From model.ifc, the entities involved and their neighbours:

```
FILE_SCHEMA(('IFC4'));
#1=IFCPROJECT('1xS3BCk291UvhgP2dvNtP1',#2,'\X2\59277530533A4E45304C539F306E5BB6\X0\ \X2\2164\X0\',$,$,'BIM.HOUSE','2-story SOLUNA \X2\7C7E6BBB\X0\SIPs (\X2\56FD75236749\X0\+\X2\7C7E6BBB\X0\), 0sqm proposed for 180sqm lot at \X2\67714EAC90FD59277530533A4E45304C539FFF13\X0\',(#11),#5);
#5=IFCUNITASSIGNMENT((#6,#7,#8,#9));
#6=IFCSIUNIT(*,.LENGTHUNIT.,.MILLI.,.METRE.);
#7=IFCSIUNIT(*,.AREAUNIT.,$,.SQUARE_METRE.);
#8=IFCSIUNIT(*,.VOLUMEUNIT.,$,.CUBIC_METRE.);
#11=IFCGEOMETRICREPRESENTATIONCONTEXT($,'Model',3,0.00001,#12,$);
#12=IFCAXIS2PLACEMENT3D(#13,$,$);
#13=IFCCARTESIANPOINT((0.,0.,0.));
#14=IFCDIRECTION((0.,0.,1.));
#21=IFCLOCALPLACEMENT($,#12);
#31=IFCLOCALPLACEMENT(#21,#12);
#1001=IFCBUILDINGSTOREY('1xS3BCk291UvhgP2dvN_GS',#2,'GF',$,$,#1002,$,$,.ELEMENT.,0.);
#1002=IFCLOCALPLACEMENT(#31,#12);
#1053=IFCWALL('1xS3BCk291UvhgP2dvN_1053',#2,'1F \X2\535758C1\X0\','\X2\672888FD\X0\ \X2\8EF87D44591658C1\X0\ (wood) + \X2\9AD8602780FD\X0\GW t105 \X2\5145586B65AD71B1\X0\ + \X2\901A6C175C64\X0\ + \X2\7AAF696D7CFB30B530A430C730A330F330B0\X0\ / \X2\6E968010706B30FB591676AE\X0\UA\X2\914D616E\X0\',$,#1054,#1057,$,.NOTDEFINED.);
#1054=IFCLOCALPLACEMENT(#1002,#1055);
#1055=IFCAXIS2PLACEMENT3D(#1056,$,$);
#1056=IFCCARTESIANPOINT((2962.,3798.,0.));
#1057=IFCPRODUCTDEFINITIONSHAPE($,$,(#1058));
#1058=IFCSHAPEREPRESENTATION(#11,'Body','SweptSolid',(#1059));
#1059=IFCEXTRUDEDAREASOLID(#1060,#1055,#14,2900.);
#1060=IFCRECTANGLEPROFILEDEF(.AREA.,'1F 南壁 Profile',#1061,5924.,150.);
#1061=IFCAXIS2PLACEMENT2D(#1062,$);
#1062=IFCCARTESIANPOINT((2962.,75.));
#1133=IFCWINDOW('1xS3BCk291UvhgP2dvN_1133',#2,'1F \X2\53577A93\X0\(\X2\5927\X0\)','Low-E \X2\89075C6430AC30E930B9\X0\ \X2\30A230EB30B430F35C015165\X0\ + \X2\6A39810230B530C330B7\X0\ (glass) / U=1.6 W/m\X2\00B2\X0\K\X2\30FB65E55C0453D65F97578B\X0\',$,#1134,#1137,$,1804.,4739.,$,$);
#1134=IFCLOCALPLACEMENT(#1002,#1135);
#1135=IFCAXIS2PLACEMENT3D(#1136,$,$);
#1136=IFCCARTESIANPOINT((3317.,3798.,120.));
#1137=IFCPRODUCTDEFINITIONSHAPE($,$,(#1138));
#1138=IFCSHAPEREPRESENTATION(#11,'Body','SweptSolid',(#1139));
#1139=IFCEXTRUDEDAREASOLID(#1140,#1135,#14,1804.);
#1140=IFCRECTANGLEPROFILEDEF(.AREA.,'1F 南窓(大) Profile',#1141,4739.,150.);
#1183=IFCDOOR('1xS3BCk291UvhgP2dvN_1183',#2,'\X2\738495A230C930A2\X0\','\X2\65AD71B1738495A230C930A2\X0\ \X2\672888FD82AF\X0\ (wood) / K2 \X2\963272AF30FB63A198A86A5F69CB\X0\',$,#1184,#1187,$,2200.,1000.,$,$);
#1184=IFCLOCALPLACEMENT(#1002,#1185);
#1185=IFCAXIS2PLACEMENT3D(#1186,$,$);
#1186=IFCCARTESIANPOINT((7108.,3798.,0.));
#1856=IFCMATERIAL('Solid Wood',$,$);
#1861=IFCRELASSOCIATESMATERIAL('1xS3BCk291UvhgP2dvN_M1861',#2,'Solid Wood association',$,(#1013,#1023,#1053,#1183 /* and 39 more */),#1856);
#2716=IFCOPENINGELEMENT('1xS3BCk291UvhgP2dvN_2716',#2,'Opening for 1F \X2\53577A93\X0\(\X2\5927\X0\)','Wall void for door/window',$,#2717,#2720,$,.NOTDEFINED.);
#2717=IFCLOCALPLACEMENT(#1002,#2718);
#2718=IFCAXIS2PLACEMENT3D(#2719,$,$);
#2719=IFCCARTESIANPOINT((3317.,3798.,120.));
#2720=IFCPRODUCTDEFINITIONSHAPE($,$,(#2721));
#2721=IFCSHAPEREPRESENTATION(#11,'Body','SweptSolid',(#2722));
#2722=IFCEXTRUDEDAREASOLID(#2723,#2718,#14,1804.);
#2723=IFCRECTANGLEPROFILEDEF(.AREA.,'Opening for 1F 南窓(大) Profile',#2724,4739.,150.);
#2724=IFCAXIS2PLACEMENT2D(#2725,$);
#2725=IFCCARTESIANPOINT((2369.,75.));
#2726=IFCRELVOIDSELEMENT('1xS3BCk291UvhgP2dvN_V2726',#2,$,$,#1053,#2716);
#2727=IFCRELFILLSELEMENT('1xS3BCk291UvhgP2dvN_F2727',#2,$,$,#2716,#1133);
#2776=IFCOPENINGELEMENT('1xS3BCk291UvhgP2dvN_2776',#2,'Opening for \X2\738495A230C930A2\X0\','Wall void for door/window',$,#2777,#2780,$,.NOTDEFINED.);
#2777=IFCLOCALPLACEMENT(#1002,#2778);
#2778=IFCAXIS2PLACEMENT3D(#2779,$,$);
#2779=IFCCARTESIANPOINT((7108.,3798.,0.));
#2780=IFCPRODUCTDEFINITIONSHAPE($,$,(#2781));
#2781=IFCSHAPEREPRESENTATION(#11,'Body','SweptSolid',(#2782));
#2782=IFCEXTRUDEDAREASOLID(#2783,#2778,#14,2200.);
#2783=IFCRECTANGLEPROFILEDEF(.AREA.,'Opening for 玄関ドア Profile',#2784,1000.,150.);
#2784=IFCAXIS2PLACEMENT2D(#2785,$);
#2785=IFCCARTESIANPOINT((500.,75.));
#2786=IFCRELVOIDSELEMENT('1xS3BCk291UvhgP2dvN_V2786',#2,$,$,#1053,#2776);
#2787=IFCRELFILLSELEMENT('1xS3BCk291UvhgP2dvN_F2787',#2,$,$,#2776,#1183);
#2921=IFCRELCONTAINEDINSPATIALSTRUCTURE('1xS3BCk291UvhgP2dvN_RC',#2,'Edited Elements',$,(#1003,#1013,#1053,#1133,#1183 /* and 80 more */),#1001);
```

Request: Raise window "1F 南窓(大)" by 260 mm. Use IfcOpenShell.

```python
import numpy as np
import ifcopenshell
import ifcopenshell.api.geometry
import ifcopenshell.util.placement
import ifcopenshell.util.unit

model = ifcopenshell.open("model.ifc")
unit_scale = ifcopenshell.util.unit.calculate_unit_scale(model)

window = model.by_guid("1xS3BCk291UvhgP2dvN_1133")
opening = window.FillsVoids[0].RelatingOpeningElement
dz = 0.26 / unit_scale

shift = np.array([0.0, 0.0, dz])
# The window is not placed relative to its opening, so move both.
for product in (opening, window):
    matrix = ifcopenshell.util.placement.get_local_placement(product.ObjectPlacement)
    matrix[:3, 3] += shift
    ifcopenshell.api.geometry.edit_object_placement(model, product=product, matrix=matrix, is_si=False)

print(f"moved by {dz * unit_scale:+.3f} m")

model.write("model-out.ifc")
```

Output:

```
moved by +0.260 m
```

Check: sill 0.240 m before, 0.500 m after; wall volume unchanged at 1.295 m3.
